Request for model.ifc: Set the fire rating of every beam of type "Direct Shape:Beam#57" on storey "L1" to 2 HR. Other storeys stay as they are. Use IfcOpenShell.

First a look at what the model holds.

```python
import ifcopenshell
import ifcopenshell.util.element

model = ifcopenshell.open("model.ifc")
print(model.schema)
storey = next(s for s in model.by_type("IfcBuildingStorey") if s.Name == "L1")
beams = [e for e in ifcopenshell.util.element.get_decomposition(storey) if e.is_a("IfcBeam")]
seen = {}
for e in beams:
    element_type = ifcopenshell.util.element.get_type(e)
    key = (element_type.Name if element_type != e and element_type else None, ifcopenshell.util.element.get_pset(e, "Pset_BeamCommon", "FireRating"))
    seen[key] = seen.get(key, 0) + 1
for (name, value), count in sorted(seen.items(), key=str):
    print(count, "x", name, "|", value)
```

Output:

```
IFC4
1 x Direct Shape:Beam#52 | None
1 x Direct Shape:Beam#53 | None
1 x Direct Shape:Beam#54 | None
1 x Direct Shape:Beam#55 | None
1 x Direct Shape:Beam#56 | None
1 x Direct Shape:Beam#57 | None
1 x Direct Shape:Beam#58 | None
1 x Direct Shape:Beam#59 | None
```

```python
import ifcopenshell
import ifcopenshell.api.pset
import ifcopenshell.util.element

model = ifcopenshell.open("model.ifc")

storey = next(s for s in model.by_type("IfcBuildingStorey") if s.Name == "L1")
beams = [e for e in ifcopenshell.util.element.get_decomposition(storey) if e.is_a("IfcBeam")]

count = 0
for e in beams:
    element_type = ifcopenshell.util.element.get_type(e)
    if element_type in (None, e) or element_type.Name != "Direct Shape:Beam#57":
        continue
    # add_pset returns the element's existing set when there is one.
    pset = ifcopenshell.api.pset.add_pset(model, product=e, name="Pset_BeamCommon")
    ifcopenshell.api.pset.edit_pset(model, pset=pset, properties={"FireRating": "2 HR"})
    count += 1

print(count, "beams updated")

model.write("model_updated.ifc")
```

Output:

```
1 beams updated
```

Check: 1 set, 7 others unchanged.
